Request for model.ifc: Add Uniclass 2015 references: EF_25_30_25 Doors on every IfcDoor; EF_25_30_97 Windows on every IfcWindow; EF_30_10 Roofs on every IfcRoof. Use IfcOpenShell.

First a look at what the model holds.

```python
import ifcopenshell

model = ifcopenshell.open("model.ifc")
print(model.schema)
print("classifications:", [c.Name for c in model.by_type("IfcClassification")])
for ifc_class in ("IfcDoor", "IfcRoof", "IfcStair", "IfcWall", "IfcWindow"):
    print(ifc_class, len(model.by_type(ifc_class)))
```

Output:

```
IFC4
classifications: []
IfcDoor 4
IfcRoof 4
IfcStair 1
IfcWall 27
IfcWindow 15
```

```python
import ifcopenshell
import ifcopenshell.api.classification

model = ifcopenshell.open("model.ifc")

system = ifcopenshell.api.classification.add_classification(model, classification="Uniclass 2015")

codes = {
    "IfcDoor": ("EF_25_30_25", "Doors"),
    "IfcWindow": ("EF_25_30_97", "Windows"),
    "IfcRoof": ("EF_30_10", "Roofs"),
}
for ifc_class, (code, name) in codes.items():
    products = model.by_type(ifc_class)
    ifcopenshell.api.classification.add_reference(
        model, products=products, classification=system, identification=code, name=name
    )
    print(code, len(products))

model.write("model_rev.ifc")
```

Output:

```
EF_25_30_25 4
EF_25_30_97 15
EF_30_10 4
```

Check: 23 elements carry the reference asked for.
